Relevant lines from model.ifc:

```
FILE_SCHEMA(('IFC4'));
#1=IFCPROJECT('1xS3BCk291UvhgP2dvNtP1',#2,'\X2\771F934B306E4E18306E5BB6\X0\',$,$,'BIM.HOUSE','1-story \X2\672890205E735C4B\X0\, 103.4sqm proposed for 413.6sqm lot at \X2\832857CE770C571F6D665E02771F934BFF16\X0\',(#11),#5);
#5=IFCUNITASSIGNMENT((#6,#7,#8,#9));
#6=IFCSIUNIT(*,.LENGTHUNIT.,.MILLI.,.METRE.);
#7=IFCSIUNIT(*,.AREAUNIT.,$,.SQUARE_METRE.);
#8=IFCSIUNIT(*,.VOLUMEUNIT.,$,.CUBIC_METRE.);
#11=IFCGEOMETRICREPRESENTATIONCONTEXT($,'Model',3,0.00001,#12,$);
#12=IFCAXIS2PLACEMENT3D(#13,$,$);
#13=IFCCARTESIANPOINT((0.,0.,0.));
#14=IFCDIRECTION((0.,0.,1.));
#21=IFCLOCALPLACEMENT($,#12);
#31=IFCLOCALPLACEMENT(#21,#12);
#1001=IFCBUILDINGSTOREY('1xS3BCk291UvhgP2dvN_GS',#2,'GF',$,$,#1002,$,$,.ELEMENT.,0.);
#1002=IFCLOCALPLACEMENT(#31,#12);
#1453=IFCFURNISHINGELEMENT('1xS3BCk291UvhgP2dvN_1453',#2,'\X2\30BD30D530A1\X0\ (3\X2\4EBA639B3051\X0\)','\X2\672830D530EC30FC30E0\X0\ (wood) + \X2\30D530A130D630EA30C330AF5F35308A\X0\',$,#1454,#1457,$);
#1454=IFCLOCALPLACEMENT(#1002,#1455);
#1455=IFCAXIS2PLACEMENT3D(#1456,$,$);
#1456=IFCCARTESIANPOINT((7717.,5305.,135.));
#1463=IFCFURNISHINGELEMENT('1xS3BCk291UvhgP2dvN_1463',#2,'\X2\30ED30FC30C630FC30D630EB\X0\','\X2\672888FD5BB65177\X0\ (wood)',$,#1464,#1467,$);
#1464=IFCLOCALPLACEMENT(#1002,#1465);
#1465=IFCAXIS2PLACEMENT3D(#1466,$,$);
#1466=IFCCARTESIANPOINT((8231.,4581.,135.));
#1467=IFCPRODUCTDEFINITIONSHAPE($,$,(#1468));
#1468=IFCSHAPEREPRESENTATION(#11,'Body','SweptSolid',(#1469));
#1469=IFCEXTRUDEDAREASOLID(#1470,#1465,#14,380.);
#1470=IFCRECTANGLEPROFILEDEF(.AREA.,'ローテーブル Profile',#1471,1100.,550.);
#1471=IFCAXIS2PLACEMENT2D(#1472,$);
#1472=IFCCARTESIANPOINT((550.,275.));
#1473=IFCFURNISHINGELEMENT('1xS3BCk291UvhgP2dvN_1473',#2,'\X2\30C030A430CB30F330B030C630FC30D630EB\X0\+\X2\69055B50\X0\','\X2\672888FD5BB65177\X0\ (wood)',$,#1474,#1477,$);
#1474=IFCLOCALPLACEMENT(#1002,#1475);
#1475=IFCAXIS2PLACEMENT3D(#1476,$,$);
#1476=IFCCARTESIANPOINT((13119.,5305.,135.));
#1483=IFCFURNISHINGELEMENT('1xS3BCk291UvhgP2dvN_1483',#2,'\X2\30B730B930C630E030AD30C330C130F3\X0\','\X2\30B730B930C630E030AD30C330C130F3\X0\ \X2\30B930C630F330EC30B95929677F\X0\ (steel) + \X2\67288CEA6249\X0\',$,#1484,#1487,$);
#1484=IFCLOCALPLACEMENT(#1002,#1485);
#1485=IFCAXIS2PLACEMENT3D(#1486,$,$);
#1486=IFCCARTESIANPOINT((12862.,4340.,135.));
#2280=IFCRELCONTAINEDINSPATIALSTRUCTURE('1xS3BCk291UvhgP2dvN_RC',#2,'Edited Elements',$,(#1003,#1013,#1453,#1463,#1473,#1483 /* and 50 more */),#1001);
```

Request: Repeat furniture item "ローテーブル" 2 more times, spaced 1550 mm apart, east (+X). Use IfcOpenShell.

```python
import numpy as np
import ifcopenshell
import ifcopenshell.api.geometry
import ifcopenshell.api.root
import ifcopenshell.util.element
import ifcopenshell.util.placement
import ifcopenshell.util.unit

model = ifcopenshell.open("model.ifc")
unit_scale = ifcopenshell.util.unit.calculate_unit_scale(model)


def reuse_history(source, copy):
    """copy_class also copies each property set's owner history, people and application; keep the originals."""
    for rel in copy.IsDefinedBy:
        if rel.is_a("IfcRelDefinesByProperties") and (history := rel.RelatingPropertyDefinition.OwnerHistory):
            rel.RelatingPropertyDefinition.OwnerHistory = source.OwnerHistory
            ifcopenshell.util.element.remove_deep2(model, history)


source = model.by_id(1463)
base = ifcopenshell.util.placement.get_local_placement(source.ObjectPlacement)
step = np.array([1.0, 0.0, 0.0]) * 1.55 / unit_scale

for i in range(1, 3):
    copy = ifcopenshell.api.root.copy_class(model, product=source)
    copy.Representation = ifcopenshell.util.element.copy_deep(
        model, source.Representation, exclude=["IfcGeometricRepresentationContext", "IfcRepresentationMap"]
    )
    reuse_history(source, copy)
    matrix = base.copy()
    matrix[:3, 3] += i * step
    print("added at", matrix[:3, 3].round(3) + 0.0)
    ifcopenshell.api.geometry.edit_object_placement(model, product=copy, matrix=matrix, is_si=False)

model.write("model_rev.ifc")
```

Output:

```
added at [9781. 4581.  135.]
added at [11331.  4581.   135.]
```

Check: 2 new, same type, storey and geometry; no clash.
